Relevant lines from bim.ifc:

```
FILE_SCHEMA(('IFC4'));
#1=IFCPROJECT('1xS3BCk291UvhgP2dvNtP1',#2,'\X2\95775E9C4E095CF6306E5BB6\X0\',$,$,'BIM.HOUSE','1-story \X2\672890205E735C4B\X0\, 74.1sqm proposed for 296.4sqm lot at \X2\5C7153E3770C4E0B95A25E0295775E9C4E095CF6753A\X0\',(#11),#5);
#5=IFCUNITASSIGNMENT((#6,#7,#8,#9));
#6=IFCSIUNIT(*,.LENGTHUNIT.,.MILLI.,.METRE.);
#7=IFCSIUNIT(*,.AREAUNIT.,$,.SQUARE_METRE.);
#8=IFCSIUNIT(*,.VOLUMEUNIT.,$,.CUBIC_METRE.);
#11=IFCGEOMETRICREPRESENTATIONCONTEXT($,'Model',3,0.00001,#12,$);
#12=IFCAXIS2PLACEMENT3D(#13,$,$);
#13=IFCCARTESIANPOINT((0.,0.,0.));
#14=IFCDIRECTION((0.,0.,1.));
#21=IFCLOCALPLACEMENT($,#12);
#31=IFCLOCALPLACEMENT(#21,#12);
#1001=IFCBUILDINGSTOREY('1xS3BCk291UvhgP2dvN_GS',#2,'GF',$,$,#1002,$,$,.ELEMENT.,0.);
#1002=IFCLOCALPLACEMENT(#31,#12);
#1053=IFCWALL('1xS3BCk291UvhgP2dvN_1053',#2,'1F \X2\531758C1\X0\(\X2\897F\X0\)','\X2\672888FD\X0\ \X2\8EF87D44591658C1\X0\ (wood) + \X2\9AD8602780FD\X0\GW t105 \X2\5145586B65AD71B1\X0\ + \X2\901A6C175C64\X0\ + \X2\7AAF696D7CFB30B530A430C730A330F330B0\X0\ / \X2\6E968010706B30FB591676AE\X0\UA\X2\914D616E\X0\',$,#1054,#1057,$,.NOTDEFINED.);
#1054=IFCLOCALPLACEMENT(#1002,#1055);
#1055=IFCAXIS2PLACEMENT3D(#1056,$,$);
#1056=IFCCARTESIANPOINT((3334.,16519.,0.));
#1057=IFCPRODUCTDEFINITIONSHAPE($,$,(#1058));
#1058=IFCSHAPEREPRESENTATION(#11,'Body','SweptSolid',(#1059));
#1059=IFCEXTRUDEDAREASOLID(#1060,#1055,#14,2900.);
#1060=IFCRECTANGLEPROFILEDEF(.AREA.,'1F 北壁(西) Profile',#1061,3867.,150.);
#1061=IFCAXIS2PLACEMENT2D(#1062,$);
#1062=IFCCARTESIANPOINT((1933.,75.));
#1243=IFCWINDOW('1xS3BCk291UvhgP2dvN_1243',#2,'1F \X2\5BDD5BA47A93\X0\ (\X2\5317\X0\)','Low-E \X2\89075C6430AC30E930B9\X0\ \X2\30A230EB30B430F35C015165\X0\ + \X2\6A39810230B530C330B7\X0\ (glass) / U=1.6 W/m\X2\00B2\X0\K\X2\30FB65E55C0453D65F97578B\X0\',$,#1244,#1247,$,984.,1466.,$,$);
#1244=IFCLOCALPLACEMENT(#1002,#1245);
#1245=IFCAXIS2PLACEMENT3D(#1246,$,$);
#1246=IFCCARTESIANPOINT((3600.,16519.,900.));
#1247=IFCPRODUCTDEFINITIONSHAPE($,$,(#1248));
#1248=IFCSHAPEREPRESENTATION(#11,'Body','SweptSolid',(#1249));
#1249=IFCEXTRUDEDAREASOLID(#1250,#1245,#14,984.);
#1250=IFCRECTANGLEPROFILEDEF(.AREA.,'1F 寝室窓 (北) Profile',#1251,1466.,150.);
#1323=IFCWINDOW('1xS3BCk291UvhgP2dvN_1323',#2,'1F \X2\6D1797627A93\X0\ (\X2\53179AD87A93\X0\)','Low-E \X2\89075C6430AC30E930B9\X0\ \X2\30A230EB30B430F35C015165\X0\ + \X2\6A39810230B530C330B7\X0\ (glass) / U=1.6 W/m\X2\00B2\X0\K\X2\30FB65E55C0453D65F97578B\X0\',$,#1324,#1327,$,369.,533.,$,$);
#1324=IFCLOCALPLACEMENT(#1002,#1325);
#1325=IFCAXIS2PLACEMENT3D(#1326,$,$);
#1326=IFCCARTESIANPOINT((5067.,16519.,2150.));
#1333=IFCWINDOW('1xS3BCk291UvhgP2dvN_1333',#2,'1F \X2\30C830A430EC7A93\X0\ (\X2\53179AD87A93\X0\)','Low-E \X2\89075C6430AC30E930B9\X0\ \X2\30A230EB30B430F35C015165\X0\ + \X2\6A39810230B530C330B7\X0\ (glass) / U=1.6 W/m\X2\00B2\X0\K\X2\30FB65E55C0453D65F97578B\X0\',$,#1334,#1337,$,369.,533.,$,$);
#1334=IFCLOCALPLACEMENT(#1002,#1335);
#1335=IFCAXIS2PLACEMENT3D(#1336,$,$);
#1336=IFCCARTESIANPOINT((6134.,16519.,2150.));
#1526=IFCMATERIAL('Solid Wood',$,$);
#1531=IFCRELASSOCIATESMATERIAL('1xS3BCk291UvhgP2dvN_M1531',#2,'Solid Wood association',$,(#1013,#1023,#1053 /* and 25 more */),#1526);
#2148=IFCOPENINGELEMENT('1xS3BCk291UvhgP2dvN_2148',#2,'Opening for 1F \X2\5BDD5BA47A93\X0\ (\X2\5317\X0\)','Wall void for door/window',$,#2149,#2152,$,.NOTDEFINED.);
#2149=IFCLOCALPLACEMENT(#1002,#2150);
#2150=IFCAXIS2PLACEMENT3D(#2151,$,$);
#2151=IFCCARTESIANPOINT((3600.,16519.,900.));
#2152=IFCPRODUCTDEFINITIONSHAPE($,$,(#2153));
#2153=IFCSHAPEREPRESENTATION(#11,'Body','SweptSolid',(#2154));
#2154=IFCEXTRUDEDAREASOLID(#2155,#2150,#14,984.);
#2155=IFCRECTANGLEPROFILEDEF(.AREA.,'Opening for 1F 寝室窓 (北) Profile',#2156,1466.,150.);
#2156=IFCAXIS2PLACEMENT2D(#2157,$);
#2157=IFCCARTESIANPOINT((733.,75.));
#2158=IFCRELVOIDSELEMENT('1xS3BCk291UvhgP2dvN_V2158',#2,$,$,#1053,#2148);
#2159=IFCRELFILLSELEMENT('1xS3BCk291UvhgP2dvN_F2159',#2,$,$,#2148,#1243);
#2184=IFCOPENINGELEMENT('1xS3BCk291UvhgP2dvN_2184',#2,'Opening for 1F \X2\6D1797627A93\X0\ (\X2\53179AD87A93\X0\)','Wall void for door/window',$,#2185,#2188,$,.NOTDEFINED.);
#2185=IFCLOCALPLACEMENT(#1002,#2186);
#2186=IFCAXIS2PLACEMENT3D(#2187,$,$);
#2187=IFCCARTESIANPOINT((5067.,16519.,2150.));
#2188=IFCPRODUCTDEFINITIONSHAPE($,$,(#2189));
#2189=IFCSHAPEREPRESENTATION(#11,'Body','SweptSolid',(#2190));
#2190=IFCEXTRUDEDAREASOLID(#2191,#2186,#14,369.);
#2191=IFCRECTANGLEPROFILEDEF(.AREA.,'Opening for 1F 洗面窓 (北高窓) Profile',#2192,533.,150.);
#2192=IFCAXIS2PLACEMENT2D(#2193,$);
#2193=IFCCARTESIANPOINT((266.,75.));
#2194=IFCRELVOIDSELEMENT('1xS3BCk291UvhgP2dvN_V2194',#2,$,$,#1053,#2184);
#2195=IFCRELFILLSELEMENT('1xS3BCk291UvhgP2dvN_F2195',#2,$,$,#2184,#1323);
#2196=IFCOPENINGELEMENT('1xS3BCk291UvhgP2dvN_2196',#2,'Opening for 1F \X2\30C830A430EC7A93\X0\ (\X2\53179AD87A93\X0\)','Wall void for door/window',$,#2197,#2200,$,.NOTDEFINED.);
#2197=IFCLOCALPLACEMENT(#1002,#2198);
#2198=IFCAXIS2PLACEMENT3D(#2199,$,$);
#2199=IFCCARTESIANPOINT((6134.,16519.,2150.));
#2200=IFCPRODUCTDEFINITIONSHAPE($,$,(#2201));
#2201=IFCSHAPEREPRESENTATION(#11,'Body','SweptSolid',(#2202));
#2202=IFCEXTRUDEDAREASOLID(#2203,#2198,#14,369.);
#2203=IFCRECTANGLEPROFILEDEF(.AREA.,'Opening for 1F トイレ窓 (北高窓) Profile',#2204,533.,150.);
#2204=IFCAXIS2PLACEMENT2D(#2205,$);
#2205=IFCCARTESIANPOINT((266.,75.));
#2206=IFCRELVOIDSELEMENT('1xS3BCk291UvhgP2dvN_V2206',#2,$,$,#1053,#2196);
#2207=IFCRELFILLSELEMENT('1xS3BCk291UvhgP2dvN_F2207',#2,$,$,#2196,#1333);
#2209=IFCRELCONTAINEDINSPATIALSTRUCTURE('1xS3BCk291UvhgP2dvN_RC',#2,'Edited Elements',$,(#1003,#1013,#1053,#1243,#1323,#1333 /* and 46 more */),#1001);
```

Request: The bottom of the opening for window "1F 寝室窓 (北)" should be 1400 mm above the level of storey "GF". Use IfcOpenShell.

```python
import numpy as np
import ifcopenshell
import ifcopenshell.api.geometry
import ifcopenshell.geom
import ifcopenshell.util.element
import ifcopenshell.util.placement
import ifcopenshell.util.shape
import ifcopenshell.util.unit

model = ifcopenshell.open("bim.ifc")
unit_scale = ifcopenshell.util.unit.calculate_unit_scale(model)

window = model.by_guid("1xS3BCk291UvhgP2dvN_1243")
opening = window.FillsVoids[0].RelatingOpeningElement
storey = ifcopenshell.util.element.get_container(window, ifc_class="IfcBuildingStorey")
level = ifcopenshell.util.placement.get_local_placement(storey.ObjectPlacement)[2, 3]

# The opening's origin need not be at the sill, so measure its lowest point.
shape = ifcopenshell.geom.create_shape(ifcopenshell.geom.settings(), opening)
bottom = ifcopenshell.util.shape.get_shape_bottom_elevation(shape, shape.geometry) / unit_scale
dz = level + 1400.0 - bottom

shift = np.array([0.0, 0.0, dz])
# The window is not placed relative to its opening, so move both.
for product in (opening, window):
    matrix = ifcopenshell.util.placement.get_local_placement(product.ObjectPlacement)
    matrix[:3, 3] += shift
    ifcopenshell.api.geometry.edit_object_placement(model, product=product, matrix=matrix, is_si=False)

print(f"moved by {dz * unit_scale:+.3f} m")

model.write("bim_v2.ifc")
```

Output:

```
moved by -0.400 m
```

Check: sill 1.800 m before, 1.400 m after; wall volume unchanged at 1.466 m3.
